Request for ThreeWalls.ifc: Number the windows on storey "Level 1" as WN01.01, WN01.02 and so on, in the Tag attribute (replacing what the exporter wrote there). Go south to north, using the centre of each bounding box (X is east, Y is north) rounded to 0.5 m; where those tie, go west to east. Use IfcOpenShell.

First a look at what the model holds.

```python
import ifcopenshell
import ifcopenshell.util.element
import ifcopenshell.util.placement

model = ifcopenshell.open("ThreeWalls.ifc")
print(model.schema)
storey = next(s for s in model.by_type("IfcBuildingStorey") if s.Name == "Level 1")
windows = [e for e in ifcopenshell.util.element.get_decomposition(storey) if e.is_a("IfcWindow")]
for e in sorted(windows, key=lambda e: e.id()):
    origin = ifcopenshell.util.placement.get_local_placement(e.ObjectPlacement)[:3, 3]
    print(e.id(), e.Tag, e.Name, origin.round(2) + 0.0, sep=" | ")
```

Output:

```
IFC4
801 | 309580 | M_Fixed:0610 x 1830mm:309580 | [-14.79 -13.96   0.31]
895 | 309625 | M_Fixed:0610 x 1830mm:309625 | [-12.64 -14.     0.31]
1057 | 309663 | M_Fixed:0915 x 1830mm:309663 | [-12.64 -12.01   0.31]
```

```python
import ifcopenshell
import ifcopenshell.geom
import ifcopenshell.util.element
import ifcopenshell.util.shape

model = ifcopenshell.open("ThreeWalls.ifc")
settings = ifcopenshell.geom.settings()
settings.set("use-world-coords", True)


def centre(element):
    shape = ifcopenshell.geom.create_shape(settings, element)
    return ifcopenshell.util.shape.get_bbox_centroid(shape.geometry)


storey = next(s for s in model.by_type("IfcBuildingStorey") if s.Name == "Level 1")
windows = [e for e in ifcopenshell.util.element.get_decomposition(storey) if e.is_a("IfcWindow")]

# Insertion points can sit at a corner or the storey origin, so sort by the geometry (in metres).
centres = {e: centre(e) for e in windows}
windows.sort(key=lambda e: (round(centres[e][1] / 0.5), centres[e][0]))

for i, e in enumerate(windows, start=1):
    number = f"WN01.{i:02d}"
    e.Tag = number
    print(e.id(), number)

model.write("ThreeWalls_edited.ifc")
```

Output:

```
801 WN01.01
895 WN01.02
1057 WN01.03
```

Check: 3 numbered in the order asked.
